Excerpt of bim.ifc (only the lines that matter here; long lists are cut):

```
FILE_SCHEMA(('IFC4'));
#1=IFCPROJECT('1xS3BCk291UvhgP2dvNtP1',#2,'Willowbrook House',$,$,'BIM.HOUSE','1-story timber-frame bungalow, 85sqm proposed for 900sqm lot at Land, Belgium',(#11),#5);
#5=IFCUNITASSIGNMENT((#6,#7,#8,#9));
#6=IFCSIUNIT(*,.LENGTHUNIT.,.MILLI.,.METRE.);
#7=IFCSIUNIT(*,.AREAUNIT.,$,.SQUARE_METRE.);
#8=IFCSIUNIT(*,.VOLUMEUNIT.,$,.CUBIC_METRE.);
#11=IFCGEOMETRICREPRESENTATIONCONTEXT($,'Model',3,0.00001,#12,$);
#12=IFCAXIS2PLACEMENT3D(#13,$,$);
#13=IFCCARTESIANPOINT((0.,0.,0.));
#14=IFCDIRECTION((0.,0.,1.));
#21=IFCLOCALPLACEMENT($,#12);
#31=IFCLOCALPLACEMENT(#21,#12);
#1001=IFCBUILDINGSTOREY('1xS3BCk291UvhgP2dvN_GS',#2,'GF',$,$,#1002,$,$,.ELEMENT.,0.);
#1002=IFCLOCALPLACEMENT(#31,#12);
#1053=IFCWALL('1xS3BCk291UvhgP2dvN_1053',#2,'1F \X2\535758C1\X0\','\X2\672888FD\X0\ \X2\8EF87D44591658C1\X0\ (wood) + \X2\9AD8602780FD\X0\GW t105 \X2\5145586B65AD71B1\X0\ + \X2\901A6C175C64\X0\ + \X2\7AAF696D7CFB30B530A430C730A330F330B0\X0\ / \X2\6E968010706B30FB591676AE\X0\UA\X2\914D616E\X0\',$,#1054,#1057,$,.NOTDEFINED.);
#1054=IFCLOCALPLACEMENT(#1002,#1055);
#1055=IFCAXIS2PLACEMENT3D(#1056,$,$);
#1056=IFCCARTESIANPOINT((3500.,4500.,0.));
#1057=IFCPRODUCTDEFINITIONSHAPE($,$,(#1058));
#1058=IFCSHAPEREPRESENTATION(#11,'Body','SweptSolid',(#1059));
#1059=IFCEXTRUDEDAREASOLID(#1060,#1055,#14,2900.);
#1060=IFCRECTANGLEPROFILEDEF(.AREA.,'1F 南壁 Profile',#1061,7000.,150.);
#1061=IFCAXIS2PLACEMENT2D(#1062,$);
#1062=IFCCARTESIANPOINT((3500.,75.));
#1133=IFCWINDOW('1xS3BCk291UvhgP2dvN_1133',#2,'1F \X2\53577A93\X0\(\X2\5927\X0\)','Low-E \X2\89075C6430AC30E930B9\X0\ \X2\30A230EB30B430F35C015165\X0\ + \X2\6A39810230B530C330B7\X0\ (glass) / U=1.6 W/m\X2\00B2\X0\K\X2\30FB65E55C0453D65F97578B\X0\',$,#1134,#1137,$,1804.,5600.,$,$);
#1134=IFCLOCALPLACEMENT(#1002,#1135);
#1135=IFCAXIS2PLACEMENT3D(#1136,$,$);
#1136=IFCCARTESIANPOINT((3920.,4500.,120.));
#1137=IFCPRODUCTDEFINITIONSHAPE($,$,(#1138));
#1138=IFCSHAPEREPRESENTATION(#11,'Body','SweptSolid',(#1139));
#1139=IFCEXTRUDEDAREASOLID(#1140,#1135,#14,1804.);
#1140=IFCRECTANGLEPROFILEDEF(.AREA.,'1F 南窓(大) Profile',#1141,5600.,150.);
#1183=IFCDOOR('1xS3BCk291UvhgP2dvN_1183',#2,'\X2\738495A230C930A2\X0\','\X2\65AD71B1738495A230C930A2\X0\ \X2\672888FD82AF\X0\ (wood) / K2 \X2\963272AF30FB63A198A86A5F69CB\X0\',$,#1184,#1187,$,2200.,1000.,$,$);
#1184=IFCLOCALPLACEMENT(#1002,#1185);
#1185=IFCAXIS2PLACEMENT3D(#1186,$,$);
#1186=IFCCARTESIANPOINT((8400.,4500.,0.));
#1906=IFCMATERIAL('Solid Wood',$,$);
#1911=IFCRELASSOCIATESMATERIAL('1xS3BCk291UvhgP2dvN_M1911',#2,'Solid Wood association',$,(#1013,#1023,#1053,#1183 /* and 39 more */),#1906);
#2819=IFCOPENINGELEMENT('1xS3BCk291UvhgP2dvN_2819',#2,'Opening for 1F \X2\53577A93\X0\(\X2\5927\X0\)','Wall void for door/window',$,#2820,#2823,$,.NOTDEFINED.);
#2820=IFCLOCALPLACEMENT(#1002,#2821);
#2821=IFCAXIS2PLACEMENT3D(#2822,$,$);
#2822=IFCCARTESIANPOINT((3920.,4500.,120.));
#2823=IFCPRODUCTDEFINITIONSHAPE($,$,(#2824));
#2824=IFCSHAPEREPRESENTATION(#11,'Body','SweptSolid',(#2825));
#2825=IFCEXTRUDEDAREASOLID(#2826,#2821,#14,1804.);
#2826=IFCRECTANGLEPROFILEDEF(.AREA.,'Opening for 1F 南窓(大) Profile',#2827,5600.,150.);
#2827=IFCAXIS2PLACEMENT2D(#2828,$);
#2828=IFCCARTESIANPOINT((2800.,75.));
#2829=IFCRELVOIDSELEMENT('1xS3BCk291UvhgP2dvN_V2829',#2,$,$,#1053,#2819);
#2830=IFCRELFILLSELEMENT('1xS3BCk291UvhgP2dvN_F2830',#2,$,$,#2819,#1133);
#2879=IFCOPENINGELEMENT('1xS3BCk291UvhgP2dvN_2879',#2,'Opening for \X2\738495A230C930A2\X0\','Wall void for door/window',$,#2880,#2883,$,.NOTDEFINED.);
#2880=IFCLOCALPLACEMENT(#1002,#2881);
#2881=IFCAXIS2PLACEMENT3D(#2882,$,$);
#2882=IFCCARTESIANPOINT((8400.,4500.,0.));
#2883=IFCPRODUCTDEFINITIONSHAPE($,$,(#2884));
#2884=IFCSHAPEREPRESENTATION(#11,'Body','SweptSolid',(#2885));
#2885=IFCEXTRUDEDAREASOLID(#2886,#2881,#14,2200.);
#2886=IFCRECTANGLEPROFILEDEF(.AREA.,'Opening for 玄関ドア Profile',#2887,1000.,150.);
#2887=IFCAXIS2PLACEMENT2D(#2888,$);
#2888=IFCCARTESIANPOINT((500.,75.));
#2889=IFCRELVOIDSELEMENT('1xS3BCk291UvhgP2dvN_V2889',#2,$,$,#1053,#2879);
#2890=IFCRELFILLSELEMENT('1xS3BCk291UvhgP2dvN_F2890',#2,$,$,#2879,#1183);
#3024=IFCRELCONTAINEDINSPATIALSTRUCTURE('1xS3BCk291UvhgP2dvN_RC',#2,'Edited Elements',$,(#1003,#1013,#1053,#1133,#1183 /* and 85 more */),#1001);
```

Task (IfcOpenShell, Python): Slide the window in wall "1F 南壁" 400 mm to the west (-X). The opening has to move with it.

```python
import ifcopenshell
import ifcopenshell.api.geometry
import ifcopenshell.util.placement

model = ifcopenshell.open("bim.ifc")

window = model.by_guid("1xS3BCk291UvhgP2dvN_1133")
opening = window.FillsVoids[0].RelatingOpeningElement
wall = opening.VoidsElements[0].RelatingBuildingElement

wall_matrix = ifcopenshell.util.placement.get_local_placement(wall.ObjectPlacement)
shift = wall_matrix[:3, 0] * -400.0
before = ifcopenshell.util.placement.get_local_placement(window.ObjectPlacement)[:3, 3].copy()

# The window is not placed relative to its opening, so move both.
for product in (opening, window):
    matrix = ifcopenshell.util.placement.get_local_placement(product.ObjectPlacement)
    matrix[:3, 3] += shift
    ifcopenshell.api.geometry.edit_object_placement(model, product=product, matrix=matrix, is_si=False)

after = ifcopenshell.util.placement.get_local_placement(window.ObjectPlacement)[:3, 3]
print("window moved by", (after - before).round(3) + 0.0)

model.write("bim_v2.ifc")
```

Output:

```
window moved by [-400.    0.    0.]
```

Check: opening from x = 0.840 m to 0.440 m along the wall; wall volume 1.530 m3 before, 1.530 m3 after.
